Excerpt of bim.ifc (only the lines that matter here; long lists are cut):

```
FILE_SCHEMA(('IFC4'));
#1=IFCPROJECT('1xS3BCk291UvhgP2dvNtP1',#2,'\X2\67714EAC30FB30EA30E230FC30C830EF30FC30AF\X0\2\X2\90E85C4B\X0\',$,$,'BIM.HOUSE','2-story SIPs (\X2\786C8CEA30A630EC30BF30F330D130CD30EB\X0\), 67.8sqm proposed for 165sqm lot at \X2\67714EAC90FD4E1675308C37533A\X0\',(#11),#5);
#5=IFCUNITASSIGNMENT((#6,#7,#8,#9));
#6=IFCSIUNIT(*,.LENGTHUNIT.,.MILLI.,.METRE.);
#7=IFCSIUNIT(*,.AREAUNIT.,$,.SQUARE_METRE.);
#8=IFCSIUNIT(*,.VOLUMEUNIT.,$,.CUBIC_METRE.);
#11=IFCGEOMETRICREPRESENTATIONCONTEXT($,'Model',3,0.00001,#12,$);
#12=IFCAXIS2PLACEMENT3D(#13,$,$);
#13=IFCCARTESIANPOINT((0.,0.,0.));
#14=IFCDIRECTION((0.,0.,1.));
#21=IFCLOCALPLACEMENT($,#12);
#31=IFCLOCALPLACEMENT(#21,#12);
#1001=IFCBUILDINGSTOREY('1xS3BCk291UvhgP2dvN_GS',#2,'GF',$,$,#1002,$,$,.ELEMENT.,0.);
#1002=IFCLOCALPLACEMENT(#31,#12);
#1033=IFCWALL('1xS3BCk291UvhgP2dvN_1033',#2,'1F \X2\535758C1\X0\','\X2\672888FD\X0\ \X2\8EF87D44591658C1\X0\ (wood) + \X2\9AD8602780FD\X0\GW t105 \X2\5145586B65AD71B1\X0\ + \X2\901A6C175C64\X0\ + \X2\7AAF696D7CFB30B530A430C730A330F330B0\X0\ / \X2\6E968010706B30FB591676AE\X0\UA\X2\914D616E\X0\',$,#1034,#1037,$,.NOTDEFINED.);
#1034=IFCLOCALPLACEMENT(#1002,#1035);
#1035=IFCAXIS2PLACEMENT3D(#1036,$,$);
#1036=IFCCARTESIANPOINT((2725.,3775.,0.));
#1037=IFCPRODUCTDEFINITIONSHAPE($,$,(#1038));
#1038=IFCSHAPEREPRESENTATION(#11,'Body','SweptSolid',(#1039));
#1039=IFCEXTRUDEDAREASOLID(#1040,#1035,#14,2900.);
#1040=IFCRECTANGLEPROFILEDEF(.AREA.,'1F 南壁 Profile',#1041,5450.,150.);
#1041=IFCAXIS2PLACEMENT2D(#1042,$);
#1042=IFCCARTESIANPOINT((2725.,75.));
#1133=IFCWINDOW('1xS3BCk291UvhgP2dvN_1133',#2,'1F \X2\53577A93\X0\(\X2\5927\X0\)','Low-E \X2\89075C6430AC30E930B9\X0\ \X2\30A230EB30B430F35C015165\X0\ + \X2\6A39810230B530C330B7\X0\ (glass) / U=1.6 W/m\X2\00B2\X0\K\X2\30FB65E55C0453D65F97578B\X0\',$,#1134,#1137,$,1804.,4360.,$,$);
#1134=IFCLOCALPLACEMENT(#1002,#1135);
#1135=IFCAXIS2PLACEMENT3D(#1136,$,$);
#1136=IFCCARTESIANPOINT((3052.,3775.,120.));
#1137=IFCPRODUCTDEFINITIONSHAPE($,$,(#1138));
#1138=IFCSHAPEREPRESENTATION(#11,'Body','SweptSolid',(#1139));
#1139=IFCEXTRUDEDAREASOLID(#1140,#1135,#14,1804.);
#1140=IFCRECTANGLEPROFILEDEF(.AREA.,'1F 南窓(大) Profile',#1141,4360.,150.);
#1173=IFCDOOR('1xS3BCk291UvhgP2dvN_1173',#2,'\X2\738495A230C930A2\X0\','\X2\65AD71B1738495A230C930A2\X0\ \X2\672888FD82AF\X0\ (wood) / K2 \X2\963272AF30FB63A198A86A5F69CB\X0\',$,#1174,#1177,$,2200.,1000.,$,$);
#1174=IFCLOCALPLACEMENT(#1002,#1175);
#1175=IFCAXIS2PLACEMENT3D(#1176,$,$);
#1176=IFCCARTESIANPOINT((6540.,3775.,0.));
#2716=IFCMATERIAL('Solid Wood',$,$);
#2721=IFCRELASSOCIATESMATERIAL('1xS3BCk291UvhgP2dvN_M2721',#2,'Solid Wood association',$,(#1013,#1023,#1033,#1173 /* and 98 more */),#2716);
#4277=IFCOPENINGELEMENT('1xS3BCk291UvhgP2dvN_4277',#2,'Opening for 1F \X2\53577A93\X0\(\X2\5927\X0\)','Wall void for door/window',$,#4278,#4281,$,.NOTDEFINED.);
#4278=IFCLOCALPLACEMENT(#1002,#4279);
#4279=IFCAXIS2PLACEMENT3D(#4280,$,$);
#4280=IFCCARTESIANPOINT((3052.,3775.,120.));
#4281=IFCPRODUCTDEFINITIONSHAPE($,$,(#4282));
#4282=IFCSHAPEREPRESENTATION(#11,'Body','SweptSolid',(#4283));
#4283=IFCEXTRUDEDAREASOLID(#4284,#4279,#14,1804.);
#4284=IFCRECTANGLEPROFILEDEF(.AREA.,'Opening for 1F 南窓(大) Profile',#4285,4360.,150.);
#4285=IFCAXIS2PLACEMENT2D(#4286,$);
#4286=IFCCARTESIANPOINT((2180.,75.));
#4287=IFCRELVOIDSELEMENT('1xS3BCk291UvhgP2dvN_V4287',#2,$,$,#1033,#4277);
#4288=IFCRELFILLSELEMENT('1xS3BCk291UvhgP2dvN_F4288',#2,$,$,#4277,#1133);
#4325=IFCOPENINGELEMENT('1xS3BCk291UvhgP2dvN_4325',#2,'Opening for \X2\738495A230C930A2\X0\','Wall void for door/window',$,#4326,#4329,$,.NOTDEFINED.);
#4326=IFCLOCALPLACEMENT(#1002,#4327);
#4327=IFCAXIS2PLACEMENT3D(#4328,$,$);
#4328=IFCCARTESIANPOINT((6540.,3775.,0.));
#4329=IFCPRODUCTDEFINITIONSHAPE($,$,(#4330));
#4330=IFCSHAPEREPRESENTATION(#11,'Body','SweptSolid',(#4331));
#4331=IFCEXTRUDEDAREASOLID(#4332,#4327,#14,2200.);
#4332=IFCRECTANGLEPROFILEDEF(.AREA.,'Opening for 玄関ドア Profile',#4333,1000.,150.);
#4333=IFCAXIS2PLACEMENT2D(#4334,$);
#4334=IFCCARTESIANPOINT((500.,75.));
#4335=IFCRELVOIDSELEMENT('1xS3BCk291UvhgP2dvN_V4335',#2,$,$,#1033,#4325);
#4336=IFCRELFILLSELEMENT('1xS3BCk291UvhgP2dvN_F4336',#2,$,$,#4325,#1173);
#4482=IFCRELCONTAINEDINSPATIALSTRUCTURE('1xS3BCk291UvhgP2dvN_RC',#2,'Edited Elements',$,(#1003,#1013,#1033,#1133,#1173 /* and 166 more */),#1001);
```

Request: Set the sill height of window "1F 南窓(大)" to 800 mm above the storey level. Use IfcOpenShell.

```python
import numpy as np
import ifcopenshell
import ifcopenshell.api.geometry
import ifcopenshell.geom
import ifcopenshell.util.element
import ifcopenshell.util.placement
import ifcopenshell.util.shape
import ifcopenshell.util.unit

model = ifcopenshell.open("bim.ifc")
unit_scale = ifcopenshell.util.unit.calculate_unit_scale(model)

window = model.by_guid("1xS3BCk291UvhgP2dvN_1133")
opening = window.FillsVoids[0].RelatingOpeningElement
storey = ifcopenshell.util.element.get_container(window, ifc_class="IfcBuildingStorey")
level = ifcopenshell.util.placement.get_local_placement(storey.ObjectPlacement)[2, 3]

# The opening's origin need not be at the sill, so measure its lowest point.
shape = ifcopenshell.geom.create_shape(ifcopenshell.geom.settings(), opening)
bottom = ifcopenshell.util.shape.get_shape_bottom_elevation(shape, shape.geometry) / unit_scale
dz = level + 800.0 - bottom

shift = np.array([0.0, 0.0, dz])
# The window is not placed relative to its opening, so move both.
for product in (opening, window):
    matrix = ifcopenshell.util.placement.get_local_placement(product.ObjectPlacement)
    matrix[:3, 3] += shift
    ifcopenshell.api.geometry.edit_object_placement(model, product=product, matrix=matrix, is_si=False)

print(f"moved by {dz * unit_scale:+.3f} m")

model.write("bim_updated.ifc")
```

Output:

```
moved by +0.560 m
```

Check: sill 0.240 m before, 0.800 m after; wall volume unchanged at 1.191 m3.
